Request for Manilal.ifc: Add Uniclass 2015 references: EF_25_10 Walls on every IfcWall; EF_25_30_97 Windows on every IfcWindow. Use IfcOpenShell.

First a look at what the model holds.

```python
import ifcopenshell

model = ifcopenshell.open("Manilal.ifc")
print(model.schema)
print("classifications:", [c.Name for c in model.by_type("IfcClassification")])
for ifc_class in ("IfcDoor", "IfcRoof", "IfcStair", "IfcWall", "IfcWindow"):
    print(ifc_class, len(model.by_type(ifc_class)))
```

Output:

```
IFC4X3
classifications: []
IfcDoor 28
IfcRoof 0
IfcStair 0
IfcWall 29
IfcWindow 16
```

```python
import ifcopenshell
import ifcopenshell.api.classification

model = ifcopenshell.open("Manilal.ifc")

system = ifcopenshell.api.classification.add_classification(model, classification="Uniclass 2015")

codes = {
    "IfcWall": ("EF_25_10", "Walls"),
    "IfcWindow": ("EF_25_30_97", "Windows"),
}
for ifc_class, (code, name) in codes.items():
    products = model.by_type(ifc_class)
    ifcopenshell.api.classification.add_reference(
        model, products=products, classification=system, identification=code, name=name
    )
    print(code, len(products))

model.write("Manilal_rev.ifc")
```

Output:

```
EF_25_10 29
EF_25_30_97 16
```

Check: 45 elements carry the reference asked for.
